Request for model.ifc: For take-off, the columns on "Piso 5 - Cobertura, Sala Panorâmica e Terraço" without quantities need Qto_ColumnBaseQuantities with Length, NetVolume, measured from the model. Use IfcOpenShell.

First a look at what the model holds.

```python
import ifcopenshell
import ifcopenshell.util.element
import ifcopenshell.util.unit

model = ifcopenshell.open("model.ifc")
print(model.schema)
for unit_type in ("LENGTHUNIT", "AREAUNIT", "VOLUMEUNIT"):
    print(unit_type, ifcopenshell.util.unit.calculate_unit_scale(model, unit_type))
storey = next(s for s in model.by_type("IfcBuildingStorey") if s.Name == "Piso 5 - Cobertura, Sala Panorâmica e Terraço")
columns = [e for e in ifcopenshell.util.element.get_decomposition(storey) if e.is_a("IfcColumn")]
for e in sorted(columns, key=lambda e: e.id()):
    print(e.id(), e.is_a(), e.Name, list(ifcopenshell.util.element.get_psets(e, qtos_only=True)), sep=" | ")
```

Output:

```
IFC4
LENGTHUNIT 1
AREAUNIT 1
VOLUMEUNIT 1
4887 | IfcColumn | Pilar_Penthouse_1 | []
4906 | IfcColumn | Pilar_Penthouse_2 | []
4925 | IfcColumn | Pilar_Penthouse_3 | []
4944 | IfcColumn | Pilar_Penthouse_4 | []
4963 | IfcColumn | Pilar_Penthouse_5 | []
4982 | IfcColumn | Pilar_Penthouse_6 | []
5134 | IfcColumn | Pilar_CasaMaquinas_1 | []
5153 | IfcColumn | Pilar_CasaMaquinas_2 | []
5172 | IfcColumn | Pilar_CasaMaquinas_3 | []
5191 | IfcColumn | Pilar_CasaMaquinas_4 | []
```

```python
import ifcopenshell
import ifcopenshell.api.pset
import ifcopenshell.geom
import ifcopenshell.util.element
import ifcopenshell.util.shape
import ifcopenshell.util.unit

model = ifcopenshell.open("model.ifc")
unit_scale = ifcopenshell.util.unit.calculate_unit_scale(model)
volume_scale = ifcopenshell.util.unit.calculate_unit_scale(model, "VOLUMEUNIT")
settings = ifcopenshell.geom.settings()

storey = next(s for s in model.by_type("IfcBuildingStorey") if s.Name == "Piso 5 - Cobertura, Sala Panorâmica e Terraço")
columns = [e for e in ifcopenshell.util.element.get_decomposition(storey) if e.is_a("IfcColumn")]

for e in sorted(columns, key=lambda e: e.id()):
    if ifcopenshell.util.element.get_psets(e, qtos_only=True, should_inherit=False):
        continue
    # Geometry comes back in metres, in the element's own axes.
    shape = ifcopenshell.geom.create_shape(settings, e)
    values = {
        "Length": ifcopenshell.util.shape.get_z(shape.geometry) / unit_scale,
        "NetVolume": ifcopenshell.util.shape.get_volume(shape.geometry) / volume_scale,
    }
    qto = ifcopenshell.api.pset.add_qto(model, product=e, name="Qto_ColumnBaseQuantities")
    ifcopenshell.api.pset.edit_qto(model, qto=qto, properties=values)
    print(e.id(), {k: round(v, 3) for k, v in values.items()})

model.write("model_updated.ifc")
```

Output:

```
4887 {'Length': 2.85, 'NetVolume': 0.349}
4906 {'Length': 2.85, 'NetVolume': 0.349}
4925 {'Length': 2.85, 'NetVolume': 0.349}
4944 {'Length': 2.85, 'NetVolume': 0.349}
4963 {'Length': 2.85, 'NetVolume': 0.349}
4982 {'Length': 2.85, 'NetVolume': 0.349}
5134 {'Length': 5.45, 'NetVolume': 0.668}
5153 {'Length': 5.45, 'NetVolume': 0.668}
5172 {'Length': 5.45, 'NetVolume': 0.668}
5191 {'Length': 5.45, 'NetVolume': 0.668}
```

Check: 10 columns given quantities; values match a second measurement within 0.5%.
